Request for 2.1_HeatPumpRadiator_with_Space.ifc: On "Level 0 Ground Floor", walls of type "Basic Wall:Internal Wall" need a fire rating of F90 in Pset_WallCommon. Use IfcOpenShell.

First a look at what the model holds.

```python
import ifcopenshell
import ifcopenshell.util.element

model = ifcopenshell.open("2.1_HeatPumpRadiator_with_Space.ifc")
print(model.schema)
storey = next(s for s in model.by_type("IfcBuildingStorey") if s.Name == "Level 0 Ground Floor")
walls = [e for e in ifcopenshell.util.element.get_decomposition(storey) if e.is_a("IfcWall")]
seen = {}
for e in walls:
    element_type = ifcopenshell.util.element.get_type(e)
    key = (element_type.Name if element_type != e and element_type else None, ifcopenshell.util.element.get_pset(e, "Pset_WallCommon", "FireRating"))
    seen[key] = seen.get(key, 0) + 1
for (name, value), count in sorted(seen.items(), key=str):
    print(count, "x", name, "|", value)
```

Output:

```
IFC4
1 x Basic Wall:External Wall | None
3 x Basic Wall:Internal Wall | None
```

```python
import ifcopenshell
import ifcopenshell.api.pset
import ifcopenshell.util.element

model = ifcopenshell.open("2.1_HeatPumpRadiator_with_Space.ifc")

storey = next(s for s in model.by_type("IfcBuildingStorey") if s.Name == "Level 0 Ground Floor")
walls = [e for e in ifcopenshell.util.element.get_decomposition(storey) if e.is_a("IfcWall")]

count = 0
for e in walls:
    element_type = ifcopenshell.util.element.get_type(e)
    if element_type in (None, e) or element_type.Name != "Basic Wall:Internal Wall":
        continue
    # add_pset returns the element's existing set when there is one.
    pset = ifcopenshell.api.pset.add_pset(model, product=e, name="Pset_WallCommon")
    ifcopenshell.api.pset.edit_pset(model, pset=pset, properties={"FireRating": "F90"})
    count += 1

print(count, "walls updated")

model.write("2.1_HeatPumpRadiator_with_Space_v2.ifc")
```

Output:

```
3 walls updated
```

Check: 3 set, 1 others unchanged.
